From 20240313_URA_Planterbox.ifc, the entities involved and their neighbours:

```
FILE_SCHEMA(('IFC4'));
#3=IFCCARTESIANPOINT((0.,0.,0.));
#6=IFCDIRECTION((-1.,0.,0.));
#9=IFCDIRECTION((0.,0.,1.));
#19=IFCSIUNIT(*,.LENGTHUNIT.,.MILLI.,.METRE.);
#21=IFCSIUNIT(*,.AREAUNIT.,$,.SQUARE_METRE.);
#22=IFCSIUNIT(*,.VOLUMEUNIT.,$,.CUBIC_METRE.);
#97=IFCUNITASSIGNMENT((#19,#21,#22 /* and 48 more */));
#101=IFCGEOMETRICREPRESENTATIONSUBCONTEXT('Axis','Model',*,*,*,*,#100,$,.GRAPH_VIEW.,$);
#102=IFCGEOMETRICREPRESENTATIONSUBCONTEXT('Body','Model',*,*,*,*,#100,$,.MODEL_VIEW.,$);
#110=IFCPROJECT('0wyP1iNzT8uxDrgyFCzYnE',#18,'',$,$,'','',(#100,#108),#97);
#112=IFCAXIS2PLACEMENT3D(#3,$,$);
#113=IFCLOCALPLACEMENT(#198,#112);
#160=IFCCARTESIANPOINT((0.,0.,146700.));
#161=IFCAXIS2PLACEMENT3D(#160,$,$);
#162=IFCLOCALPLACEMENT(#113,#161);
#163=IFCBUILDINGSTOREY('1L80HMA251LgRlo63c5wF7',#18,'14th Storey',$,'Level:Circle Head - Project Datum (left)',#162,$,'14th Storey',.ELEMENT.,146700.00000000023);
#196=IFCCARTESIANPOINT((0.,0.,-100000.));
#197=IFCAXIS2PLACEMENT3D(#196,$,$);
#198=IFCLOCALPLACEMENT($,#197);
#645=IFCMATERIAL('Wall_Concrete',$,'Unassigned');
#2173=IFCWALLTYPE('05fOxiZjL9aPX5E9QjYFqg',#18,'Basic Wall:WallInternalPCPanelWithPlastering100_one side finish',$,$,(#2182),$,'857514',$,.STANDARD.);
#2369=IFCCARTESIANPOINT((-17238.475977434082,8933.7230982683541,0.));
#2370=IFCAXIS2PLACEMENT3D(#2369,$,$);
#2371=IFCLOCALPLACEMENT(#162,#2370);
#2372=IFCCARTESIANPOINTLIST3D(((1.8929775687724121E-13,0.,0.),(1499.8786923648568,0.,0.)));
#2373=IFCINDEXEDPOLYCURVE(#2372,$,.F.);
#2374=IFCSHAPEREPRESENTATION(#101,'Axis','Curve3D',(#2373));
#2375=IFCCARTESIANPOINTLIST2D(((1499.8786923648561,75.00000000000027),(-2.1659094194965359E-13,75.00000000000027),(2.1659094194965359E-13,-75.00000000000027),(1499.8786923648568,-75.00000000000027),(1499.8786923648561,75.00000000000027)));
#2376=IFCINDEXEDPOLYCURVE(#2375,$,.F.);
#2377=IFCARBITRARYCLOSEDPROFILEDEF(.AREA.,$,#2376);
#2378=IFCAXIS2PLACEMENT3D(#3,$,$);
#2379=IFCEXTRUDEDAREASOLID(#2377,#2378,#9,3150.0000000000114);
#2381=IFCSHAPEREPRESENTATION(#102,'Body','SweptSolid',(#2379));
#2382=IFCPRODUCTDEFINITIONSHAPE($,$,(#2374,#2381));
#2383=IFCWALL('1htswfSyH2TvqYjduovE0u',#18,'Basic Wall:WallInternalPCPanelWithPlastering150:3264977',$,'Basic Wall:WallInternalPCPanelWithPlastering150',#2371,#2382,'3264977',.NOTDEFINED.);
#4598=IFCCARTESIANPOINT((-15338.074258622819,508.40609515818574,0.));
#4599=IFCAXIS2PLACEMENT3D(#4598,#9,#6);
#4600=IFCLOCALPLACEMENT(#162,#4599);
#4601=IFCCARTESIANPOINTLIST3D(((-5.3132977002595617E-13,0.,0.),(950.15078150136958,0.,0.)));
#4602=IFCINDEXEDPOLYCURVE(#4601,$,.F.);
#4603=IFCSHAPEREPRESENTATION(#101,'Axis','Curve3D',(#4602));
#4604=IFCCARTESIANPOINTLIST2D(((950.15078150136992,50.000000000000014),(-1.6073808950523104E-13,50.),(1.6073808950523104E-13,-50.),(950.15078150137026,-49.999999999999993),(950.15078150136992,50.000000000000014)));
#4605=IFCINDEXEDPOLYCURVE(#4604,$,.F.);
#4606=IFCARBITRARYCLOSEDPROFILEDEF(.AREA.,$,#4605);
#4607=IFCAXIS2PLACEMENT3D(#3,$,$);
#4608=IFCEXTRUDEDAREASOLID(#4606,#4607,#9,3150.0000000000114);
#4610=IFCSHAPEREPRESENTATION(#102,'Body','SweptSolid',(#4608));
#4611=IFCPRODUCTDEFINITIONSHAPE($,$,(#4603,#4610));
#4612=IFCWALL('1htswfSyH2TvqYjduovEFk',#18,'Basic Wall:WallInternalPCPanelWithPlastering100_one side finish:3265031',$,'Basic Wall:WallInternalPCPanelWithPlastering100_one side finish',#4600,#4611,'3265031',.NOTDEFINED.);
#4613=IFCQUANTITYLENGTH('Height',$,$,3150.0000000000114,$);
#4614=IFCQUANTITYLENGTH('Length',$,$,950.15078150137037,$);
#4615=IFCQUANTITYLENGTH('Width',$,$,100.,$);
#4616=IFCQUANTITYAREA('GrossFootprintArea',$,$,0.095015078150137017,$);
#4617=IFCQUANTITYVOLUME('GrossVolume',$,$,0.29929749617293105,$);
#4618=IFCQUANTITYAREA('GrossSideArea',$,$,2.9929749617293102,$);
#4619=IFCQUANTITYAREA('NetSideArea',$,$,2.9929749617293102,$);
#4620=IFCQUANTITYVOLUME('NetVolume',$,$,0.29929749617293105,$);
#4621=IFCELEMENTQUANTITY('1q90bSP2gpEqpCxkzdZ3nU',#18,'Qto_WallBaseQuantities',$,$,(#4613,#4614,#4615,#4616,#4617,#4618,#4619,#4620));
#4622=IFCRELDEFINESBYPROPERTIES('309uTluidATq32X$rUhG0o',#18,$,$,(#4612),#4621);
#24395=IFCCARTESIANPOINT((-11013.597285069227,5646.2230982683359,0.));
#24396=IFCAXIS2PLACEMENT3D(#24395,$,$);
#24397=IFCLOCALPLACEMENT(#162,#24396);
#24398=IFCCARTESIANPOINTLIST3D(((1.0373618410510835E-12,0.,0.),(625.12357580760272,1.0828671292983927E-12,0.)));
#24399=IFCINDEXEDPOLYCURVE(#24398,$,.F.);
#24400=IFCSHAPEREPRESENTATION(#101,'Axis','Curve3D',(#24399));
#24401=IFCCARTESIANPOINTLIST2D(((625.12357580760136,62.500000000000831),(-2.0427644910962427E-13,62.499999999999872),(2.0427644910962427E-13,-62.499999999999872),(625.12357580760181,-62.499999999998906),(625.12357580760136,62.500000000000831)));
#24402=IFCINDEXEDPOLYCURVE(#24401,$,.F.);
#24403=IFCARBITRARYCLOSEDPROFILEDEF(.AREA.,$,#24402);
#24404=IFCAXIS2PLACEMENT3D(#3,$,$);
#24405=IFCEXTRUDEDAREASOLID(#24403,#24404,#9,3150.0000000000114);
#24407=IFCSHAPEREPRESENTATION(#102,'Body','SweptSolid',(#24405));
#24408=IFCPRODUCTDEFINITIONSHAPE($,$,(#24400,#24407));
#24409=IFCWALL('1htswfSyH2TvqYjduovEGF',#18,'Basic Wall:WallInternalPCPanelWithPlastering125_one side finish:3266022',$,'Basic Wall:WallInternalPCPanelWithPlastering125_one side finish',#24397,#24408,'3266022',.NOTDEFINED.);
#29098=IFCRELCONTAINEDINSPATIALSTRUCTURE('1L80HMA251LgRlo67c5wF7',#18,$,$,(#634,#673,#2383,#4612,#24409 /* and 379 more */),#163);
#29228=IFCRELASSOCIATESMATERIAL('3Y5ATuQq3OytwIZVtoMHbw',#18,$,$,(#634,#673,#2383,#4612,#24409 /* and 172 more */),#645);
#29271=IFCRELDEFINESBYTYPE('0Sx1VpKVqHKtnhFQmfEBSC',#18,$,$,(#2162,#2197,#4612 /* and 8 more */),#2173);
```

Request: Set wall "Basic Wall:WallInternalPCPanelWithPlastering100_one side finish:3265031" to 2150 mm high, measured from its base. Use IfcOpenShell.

```python
import ifcopenshell
import ifcopenshell.api.pset
import ifcopenshell.geom
import ifcopenshell.util.element
import ifcopenshell.util.representation
import ifcopenshell.util.shape
import ifcopenshell.util.unit

model = ifcopenshell.open("20240313_URA_Planterbox.ifc")
unit_scale = ifcopenshell.util.unit.calculate_unit_scale(model)
area_scale = ifcopenshell.util.unit.calculate_unit_scale(model, "AREAUNIT")
volume_scale = ifcopenshell.util.unit.calculate_unit_scale(model, "VOLUMEUNIT")
settings = ifcopenshell.geom.settings()


def volume(element):
    """Net volume in cubic metres, openings subtracted."""
    shape = ifcopenshell.geom.create_shape(settings, element)
    return ifcopenshell.util.shape.get_volume(shape.geometry)


wall = model.by_id(4612)
before = volume(wall)

body = ifcopenshell.util.representation.get_representation(wall, "Model", "Body")
solid = body.Items[0]
old_height = solid.Depth
solid.Depth = 2150.0
after = volume(wall)
thickness = 0.1  # wall thickness in metres

# Update the stored height, areas and volumes.
qto = model.by_id(ifcopenshell.util.element.get_pset(wall, "Qto_WallBaseQuantities", should_inherit=False)["id"])
ifcopenshell.api.pset.edit_qto(model, qto=qto, properties={
    "Height": solid.Depth,
    "GrossVolume": ifcopenshell.util.element.get_pset(wall, "Qto_WallBaseQuantities", "GrossVolume") * solid.Depth / old_height,
    "GrossSideArea": ifcopenshell.util.element.get_pset(wall, "Qto_WallBaseQuantities", "GrossSideArea") * solid.Depth / old_height,
    "NetSideArea": after / thickness / area_scale,
    "NetVolume": after / volume_scale,
})

print(f"height {old_height:g} -> {solid.Depth:g}, volume {before:.3f} -> {after:.3f} m3")

model.write("20240313_URA_Planterbox-out.ifc")
```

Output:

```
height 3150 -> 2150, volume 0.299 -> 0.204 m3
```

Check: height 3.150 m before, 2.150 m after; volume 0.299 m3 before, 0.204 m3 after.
